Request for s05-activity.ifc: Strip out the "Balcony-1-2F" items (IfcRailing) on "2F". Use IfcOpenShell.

First a look at what the model holds.

```python
import ifcopenshell
import ifcopenshell.util.element

model = ifcopenshell.open("s05-activity.ifc")
print(model.schema)
storey = next(s for s in model.by_type("IfcBuildingStorey") if s.Name == "2F")
railings = [e for e in ifcopenshell.util.element.get_decomposition(storey) if e.is_a("IfcRailing")]
seen = {}
for e in railings:
    element_type = ifcopenshell.util.element.get_type(e)
    name = element_type.Name if element_type not in (None, e) else None
    seen[name] = seen.get(name, 0) + 1
for name, count in sorted(seen.items(), key=str):
    print(count, "x", name)
```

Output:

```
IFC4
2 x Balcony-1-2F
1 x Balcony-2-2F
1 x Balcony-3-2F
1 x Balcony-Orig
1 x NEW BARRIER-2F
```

```python
import ifcopenshell
import ifcopenshell.api.root
import ifcopenshell.util.element

model = ifcopenshell.open("s05-activity.ifc")

storey = next(s for s in model.by_type("IfcBuildingStorey") if s.Name == "2F")
railings = [e for e in ifcopenshell.util.element.get_decomposition(storey) if e.is_a("IfcRailing")]
targets = [e for e in railings if (t := ifcopenshell.util.element.get_type(e)) not in (None, e) and t.Name == "Balcony-1-2F"]

for e in targets:
    ifcopenshell.api.root.remove_product(model, product=e)
print(len(targets), "removed")

model.write("s05-activity_rev.ifc")
```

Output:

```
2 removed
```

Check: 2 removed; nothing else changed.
